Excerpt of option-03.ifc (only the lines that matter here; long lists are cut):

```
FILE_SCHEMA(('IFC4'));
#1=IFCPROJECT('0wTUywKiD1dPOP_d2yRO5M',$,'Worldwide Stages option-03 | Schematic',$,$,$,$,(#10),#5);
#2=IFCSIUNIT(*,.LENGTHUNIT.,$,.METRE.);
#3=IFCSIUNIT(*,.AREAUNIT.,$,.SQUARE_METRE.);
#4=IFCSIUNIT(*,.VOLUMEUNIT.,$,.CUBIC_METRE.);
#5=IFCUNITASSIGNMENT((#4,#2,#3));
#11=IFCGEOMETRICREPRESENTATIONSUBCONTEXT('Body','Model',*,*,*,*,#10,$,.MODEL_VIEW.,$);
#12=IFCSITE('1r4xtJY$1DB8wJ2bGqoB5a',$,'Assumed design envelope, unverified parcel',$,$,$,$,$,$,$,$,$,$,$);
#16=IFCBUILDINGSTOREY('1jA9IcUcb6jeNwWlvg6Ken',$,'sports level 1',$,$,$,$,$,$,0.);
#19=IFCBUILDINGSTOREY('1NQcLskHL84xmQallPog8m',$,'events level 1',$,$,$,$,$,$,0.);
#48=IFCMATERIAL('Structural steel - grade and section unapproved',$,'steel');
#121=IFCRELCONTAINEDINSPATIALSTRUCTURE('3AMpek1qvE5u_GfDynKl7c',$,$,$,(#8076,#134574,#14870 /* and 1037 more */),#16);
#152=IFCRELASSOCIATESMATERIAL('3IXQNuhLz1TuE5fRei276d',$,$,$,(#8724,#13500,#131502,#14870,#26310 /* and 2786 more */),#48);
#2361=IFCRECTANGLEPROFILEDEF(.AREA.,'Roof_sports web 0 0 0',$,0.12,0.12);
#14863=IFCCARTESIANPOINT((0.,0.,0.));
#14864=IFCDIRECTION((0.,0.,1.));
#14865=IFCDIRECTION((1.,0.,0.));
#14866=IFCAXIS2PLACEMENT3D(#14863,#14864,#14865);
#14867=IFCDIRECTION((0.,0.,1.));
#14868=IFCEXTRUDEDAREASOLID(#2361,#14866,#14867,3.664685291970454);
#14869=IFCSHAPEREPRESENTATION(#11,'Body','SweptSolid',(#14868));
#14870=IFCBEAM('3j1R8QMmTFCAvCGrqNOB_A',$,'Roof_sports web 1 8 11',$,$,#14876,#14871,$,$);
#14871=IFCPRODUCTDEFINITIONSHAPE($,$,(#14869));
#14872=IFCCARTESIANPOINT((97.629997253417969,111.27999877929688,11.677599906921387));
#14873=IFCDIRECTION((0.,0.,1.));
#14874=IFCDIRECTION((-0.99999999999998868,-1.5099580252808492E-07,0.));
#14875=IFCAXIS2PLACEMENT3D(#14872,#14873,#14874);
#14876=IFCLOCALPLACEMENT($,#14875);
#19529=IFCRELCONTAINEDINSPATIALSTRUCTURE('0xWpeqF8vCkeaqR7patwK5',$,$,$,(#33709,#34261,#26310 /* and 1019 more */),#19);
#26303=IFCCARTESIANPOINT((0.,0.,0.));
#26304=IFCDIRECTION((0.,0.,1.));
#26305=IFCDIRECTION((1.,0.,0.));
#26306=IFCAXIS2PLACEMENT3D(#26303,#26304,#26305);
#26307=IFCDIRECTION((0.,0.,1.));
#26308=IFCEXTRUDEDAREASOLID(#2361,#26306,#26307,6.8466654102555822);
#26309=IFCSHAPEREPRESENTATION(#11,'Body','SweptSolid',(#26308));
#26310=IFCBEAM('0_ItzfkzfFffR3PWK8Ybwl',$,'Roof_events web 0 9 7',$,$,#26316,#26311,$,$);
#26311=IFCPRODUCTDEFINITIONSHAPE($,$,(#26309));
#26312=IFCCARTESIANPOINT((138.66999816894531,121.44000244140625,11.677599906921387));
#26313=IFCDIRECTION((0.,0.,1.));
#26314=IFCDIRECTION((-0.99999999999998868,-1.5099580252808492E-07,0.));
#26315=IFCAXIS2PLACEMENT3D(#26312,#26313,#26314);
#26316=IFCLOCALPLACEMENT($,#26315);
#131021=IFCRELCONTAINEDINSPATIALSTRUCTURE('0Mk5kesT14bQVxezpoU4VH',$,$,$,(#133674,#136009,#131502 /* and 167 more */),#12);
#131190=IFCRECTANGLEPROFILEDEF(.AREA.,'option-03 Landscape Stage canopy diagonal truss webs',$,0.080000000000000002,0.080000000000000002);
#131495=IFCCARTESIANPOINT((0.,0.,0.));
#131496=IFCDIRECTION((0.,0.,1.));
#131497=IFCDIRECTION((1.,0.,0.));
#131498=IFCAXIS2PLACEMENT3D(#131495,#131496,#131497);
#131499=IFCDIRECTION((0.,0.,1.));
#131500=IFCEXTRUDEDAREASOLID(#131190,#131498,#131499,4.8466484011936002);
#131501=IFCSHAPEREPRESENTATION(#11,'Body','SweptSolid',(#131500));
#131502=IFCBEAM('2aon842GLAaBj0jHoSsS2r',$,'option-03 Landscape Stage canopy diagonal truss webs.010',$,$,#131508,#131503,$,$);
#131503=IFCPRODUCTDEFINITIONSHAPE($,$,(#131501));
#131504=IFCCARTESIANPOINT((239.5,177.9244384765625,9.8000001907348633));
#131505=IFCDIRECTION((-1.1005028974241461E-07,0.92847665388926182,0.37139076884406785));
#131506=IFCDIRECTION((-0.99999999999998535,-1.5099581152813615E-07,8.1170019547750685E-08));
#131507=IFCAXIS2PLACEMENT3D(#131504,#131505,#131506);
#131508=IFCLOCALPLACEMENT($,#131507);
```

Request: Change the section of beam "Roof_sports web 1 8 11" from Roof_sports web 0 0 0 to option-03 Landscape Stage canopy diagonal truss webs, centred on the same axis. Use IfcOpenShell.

```python
import ifcopenshell
import ifcopenshell.util.element
import ifcopenshell.util.representation

model = ifcopenshell.open("option-03.ifc")

member = model.by_guid("3j1R8QMmTFCAvCGrqNOB_A")
source = next(p for p in model.by_type("IfcRectangleProfileDef") if p.ProfileName == "option-03 Landscape Stage canopy diagonal truss webs")

body = ifcopenshell.util.representation.get_representation(member, "Model", "Body")
solid = body.Items[0]
old_profile = solid.SweptArea

# Copy the section's sizes but keep this member's own profile position.
profile = ifcopenshell.util.element.copy(model, source)
profile.Position = old_profile.Position
solid.SweptArea = profile
if not model.get_total_inverses(old_profile):
    ifcopenshell.util.element.remove_deep2(model, old_profile)

print(solid.SweptArea)

model.write("option-03_v2.ifc")
```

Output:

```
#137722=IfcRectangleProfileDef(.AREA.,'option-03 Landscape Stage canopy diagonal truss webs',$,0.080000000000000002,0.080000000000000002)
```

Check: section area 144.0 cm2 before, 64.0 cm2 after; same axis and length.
